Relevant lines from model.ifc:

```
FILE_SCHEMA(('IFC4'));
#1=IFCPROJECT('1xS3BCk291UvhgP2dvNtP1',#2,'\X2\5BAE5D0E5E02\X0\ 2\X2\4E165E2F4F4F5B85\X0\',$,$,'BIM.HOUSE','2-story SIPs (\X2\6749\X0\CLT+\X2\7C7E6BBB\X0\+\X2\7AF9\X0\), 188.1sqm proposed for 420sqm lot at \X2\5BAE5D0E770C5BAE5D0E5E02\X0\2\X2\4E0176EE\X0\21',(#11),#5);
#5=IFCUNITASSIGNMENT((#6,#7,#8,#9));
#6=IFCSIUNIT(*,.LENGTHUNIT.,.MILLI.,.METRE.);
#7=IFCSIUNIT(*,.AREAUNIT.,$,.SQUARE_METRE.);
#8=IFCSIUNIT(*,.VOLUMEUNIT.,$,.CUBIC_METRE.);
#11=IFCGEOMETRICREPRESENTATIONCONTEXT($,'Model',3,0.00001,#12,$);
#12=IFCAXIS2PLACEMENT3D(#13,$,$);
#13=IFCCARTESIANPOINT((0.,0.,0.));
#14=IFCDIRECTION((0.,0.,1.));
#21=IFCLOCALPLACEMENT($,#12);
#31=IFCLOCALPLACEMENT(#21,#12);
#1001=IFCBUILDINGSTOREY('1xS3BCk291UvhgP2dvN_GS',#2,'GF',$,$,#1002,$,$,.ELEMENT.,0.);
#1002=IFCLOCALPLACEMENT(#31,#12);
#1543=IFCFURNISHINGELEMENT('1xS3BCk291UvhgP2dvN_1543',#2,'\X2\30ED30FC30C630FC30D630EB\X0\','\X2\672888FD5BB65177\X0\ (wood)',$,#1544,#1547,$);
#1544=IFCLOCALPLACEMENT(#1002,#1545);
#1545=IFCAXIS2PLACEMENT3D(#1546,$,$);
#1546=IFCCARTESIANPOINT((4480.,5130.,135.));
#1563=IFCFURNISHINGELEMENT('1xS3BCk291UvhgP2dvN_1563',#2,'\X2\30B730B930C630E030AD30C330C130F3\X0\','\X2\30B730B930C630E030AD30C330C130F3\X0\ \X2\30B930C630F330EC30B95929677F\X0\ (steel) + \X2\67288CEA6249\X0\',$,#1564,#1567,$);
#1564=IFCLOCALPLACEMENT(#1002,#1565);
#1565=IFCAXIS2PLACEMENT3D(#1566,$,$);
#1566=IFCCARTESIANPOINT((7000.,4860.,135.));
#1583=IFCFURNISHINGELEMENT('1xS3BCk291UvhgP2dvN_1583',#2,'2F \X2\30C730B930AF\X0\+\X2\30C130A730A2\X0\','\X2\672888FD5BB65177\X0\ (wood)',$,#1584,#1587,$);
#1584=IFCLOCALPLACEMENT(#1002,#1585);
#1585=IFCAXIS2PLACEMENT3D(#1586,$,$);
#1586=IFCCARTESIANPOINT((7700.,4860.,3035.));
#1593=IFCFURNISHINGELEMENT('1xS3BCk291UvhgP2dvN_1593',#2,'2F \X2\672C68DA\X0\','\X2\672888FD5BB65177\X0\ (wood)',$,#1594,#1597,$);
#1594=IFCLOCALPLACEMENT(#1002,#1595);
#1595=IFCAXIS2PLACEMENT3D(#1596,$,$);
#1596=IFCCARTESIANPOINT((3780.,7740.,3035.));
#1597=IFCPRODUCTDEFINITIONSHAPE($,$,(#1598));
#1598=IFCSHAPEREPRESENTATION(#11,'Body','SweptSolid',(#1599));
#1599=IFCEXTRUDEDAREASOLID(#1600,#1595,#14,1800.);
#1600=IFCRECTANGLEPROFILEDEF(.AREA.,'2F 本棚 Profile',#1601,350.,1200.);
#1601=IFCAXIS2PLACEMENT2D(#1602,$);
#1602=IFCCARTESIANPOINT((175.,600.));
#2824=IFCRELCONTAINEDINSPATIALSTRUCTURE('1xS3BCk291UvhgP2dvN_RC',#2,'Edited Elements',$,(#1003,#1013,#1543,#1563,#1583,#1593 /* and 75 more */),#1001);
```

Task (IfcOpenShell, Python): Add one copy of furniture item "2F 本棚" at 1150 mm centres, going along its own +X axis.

```python
import ifcopenshell
import ifcopenshell.api.geometry
import ifcopenshell.api.root
import ifcopenshell.util.element
import ifcopenshell.util.placement
import ifcopenshell.util.unit

model = ifcopenshell.open("model.ifc")
unit_scale = ifcopenshell.util.unit.calculate_unit_scale(model)


def reuse_history(source, copy):
    """copy_class also copies each property set's owner history, people and application; keep the originals."""
    for rel in copy.IsDefinedBy:
        if rel.is_a("IfcRelDefinesByProperties") and (history := rel.RelatingPropertyDefinition.OwnerHistory):
            rel.RelatingPropertyDefinition.OwnerHistory = source.OwnerHistory
            ifcopenshell.util.element.remove_deep2(model, history)


source = model.by_guid("1xS3BCk291UvhgP2dvN_1593")
base = ifcopenshell.util.placement.get_local_placement(source.ObjectPlacement)
step = base[:3, 0] * 1.15 / unit_scale

for i in range(1, 2):
    copy = ifcopenshell.api.root.copy_class(model, product=source)
    copy.Representation = ifcopenshell.util.element.copy_deep(
        model, source.Representation, exclude=["IfcGeometricRepresentationContext", "IfcRepresentationMap"]
    )
    reuse_history(source, copy)
    matrix = base.copy()
    matrix[:3, 3] += i * step
    print("added at", matrix[:3, 3].round(3) + 0.0)
    ifcopenshell.api.geometry.edit_object_placement(model, product=copy, matrix=matrix, is_si=False)

model.write("model_v2.ifc")
```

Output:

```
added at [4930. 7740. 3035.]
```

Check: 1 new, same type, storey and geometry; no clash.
